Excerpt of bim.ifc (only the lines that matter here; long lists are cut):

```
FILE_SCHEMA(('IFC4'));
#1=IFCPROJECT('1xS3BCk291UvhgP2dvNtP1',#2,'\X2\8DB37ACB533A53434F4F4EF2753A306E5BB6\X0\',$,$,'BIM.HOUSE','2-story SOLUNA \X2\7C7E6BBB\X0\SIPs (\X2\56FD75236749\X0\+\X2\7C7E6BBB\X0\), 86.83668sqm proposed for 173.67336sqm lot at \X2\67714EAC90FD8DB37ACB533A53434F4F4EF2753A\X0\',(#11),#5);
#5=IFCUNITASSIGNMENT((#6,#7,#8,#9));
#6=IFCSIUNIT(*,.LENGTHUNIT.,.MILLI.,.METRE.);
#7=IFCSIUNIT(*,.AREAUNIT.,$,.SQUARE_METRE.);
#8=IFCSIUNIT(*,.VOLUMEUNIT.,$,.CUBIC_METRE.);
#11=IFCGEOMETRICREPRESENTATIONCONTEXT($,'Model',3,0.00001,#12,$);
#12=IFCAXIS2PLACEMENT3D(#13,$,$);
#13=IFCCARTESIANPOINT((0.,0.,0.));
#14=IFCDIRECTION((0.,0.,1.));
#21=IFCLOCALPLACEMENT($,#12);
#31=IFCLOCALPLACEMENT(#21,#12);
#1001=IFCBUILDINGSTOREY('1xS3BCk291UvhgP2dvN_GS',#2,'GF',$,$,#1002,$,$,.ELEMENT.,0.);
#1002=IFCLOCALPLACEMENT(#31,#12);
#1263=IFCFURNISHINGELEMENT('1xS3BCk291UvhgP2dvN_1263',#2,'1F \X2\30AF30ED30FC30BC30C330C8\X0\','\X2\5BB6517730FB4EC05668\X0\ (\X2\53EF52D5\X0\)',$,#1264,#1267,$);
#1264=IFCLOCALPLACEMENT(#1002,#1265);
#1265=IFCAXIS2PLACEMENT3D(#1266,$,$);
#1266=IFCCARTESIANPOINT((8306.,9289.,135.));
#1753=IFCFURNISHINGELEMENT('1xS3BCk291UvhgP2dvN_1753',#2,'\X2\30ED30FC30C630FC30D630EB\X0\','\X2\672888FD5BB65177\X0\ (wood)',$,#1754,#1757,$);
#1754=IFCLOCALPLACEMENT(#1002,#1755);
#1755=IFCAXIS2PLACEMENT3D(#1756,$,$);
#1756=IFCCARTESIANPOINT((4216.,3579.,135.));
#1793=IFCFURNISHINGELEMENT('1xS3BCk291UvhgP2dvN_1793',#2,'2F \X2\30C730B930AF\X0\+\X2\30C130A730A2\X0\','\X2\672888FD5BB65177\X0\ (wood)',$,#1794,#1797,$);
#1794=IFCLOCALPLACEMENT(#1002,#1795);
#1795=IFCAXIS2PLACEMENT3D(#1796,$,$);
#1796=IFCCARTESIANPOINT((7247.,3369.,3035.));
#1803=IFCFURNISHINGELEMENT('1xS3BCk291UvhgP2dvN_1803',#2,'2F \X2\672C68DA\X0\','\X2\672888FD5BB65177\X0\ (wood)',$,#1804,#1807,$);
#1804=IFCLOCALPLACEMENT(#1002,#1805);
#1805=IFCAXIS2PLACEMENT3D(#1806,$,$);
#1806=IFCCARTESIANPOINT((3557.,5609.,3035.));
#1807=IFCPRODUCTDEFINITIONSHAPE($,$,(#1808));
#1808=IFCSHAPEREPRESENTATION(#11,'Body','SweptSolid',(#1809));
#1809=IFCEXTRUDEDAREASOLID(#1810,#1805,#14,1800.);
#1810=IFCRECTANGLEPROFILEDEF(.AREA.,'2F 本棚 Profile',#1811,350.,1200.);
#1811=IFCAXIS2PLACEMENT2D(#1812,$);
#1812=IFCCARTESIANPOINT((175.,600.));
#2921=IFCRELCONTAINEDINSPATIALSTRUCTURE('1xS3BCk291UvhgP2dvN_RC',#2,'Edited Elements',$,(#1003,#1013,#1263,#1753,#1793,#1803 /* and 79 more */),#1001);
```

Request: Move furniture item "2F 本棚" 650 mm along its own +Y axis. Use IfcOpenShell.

```python
import ifcopenshell
import ifcopenshell.api.geometry
import ifcopenshell.util.placement
import ifcopenshell.util.unit

model = ifcopenshell.open("bim.ifc")
unit_scale = ifcopenshell.util.unit.calculate_unit_scale(model)

item = model.by_id(1803)
matrix = ifcopenshell.util.placement.get_local_placement(item.ObjectPlacement)
matrix[:3, 3] += matrix[:3, 1] * 0.65 / unit_scale
ifcopenshell.api.geometry.edit_object_placement(model, product=item, matrix=matrix, is_si=False)

print(ifcopenshell.util.placement.get_local_placement(item.ObjectPlacement).round(3) + 0.0)

model.write("bim_rev.ifc")
```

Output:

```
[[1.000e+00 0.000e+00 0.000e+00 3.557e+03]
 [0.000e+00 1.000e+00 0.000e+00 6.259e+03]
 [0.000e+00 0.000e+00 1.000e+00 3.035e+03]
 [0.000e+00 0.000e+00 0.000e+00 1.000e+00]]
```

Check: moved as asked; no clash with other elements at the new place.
